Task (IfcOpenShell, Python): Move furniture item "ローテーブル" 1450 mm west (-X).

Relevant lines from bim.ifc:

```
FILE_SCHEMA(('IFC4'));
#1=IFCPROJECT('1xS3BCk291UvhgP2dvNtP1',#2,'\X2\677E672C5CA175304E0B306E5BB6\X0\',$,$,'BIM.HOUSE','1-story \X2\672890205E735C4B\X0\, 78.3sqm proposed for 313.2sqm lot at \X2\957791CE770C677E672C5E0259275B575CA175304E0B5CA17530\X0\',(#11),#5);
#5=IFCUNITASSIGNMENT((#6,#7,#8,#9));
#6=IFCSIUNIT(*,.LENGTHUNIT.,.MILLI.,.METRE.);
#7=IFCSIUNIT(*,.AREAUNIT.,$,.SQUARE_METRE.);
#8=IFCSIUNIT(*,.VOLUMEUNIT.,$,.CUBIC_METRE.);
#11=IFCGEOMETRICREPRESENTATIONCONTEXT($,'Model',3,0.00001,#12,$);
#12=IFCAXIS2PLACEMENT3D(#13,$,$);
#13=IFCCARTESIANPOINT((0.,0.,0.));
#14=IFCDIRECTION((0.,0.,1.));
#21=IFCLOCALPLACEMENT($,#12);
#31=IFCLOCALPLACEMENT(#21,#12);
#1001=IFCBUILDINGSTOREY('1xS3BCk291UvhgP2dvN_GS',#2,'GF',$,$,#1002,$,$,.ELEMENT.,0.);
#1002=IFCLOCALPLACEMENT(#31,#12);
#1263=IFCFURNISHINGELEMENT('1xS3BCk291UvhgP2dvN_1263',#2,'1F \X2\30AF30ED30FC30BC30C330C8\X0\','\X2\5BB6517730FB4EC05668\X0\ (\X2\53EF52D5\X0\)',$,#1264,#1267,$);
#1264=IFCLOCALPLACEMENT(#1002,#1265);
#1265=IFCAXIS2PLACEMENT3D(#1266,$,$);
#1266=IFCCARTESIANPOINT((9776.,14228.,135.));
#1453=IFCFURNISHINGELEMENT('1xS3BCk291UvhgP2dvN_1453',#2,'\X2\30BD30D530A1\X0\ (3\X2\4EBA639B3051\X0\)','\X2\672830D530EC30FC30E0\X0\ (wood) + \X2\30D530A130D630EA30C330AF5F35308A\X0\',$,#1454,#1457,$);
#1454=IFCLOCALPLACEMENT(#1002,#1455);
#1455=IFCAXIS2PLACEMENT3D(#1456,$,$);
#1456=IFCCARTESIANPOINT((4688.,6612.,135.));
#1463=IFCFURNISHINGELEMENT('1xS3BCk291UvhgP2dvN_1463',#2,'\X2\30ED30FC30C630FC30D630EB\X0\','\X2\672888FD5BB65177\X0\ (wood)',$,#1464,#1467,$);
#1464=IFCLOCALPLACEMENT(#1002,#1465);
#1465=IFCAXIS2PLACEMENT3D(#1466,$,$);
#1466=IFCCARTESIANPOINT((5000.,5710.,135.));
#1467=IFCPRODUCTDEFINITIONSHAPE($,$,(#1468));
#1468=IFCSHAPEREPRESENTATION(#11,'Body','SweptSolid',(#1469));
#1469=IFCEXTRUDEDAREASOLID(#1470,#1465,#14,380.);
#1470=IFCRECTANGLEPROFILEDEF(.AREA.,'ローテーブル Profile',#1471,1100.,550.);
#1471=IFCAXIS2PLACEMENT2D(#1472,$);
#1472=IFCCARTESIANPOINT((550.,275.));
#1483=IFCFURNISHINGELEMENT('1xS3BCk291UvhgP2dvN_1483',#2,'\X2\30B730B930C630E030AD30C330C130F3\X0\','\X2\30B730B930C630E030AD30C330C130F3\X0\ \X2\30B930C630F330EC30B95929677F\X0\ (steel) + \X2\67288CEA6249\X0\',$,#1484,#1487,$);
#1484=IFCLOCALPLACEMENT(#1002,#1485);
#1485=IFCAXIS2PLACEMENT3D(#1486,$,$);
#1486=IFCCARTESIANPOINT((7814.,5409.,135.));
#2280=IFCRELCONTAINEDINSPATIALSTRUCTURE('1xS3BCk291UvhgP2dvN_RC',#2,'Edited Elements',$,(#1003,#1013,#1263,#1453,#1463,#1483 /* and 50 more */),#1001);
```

```python
import ifcopenshell
import ifcopenshell.api.geometry
import ifcopenshell.util.placement

model = ifcopenshell.open("bim.ifc")

item = model.by_guid("1xS3BCk291UvhgP2dvN_1463")
matrix = ifcopenshell.util.placement.get_local_placement(item.ObjectPlacement)
matrix[0, 3] -= 1450.0
ifcopenshell.api.geometry.edit_object_placement(model, product=item, matrix=matrix, is_si=False)

print(ifcopenshell.util.placement.get_local_placement(item.ObjectPlacement).round(3) + 0.0)

model.write("bim-out.ifc")
```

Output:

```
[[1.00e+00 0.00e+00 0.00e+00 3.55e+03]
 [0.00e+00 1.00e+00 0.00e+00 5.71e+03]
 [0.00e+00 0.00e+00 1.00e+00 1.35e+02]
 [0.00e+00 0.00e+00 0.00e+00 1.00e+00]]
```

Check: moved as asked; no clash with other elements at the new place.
